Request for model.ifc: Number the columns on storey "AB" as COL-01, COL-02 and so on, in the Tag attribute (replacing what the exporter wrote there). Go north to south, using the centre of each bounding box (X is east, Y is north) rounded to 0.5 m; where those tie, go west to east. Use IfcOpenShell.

First a look at what the model holds.

```python
import ifcopenshell
import ifcopenshell.util.element
import ifcopenshell.util.placement

model = ifcopenshell.open("model.ifc")
print(model.schema)
storey = next(s for s in model.by_type("IfcBuildingStorey") if s.Name == "AB")
columns = [e for e in ifcopenshell.util.element.get_decomposition(storey) if e.is_a("IfcColumn")]
for e in sorted(columns, key=lambda e: e.id()):
    origin = ifcopenshell.util.placement.get_local_placement(e.ObjectPlacement)[:3, 3]
    print(e.id(), e.Tag, e.Name, origin.round(2) + 0.0, sep=" | ")
```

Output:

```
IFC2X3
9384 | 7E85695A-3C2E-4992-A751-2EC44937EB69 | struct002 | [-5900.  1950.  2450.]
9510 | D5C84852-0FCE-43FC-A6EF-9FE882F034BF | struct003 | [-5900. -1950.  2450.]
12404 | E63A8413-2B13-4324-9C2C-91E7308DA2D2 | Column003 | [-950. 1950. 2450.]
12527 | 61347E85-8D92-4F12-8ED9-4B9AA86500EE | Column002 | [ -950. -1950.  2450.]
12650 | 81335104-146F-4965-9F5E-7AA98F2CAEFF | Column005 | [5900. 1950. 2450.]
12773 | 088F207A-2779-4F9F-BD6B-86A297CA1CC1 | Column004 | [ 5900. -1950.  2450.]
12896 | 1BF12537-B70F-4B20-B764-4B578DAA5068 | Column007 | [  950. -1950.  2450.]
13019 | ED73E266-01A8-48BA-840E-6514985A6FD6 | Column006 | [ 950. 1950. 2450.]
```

```python
import ifcopenshell
import ifcopenshell.geom
import ifcopenshell.util.element
import ifcopenshell.util.shape

model = ifcopenshell.open("model.ifc")
settings = ifcopenshell.geom.settings()
settings.set("use-world-coords", True)


def centre(element):
    shape = ifcopenshell.geom.create_shape(settings, element)
    return ifcopenshell.util.shape.get_bbox_centroid(shape.geometry)


storey = next(s for s in model.by_type("IfcBuildingStorey") if s.Name == "AB")
columns = [e for e in ifcopenshell.util.element.get_decomposition(storey) if e.is_a("IfcColumn")]

# Insertion points can sit at a corner or the storey origin, so sort by the geometry (in metres).
centres = {e: centre(e) for e in columns}
columns.sort(key=lambda e: (-round(centres[e][1] / 0.5), centres[e][0]))

for i, e in enumerate(columns, start=1):
    number = f"COL-{i:02d}"
    e.Tag = number
    print(e.id(), number)

model.write("model_v2.ifc")
```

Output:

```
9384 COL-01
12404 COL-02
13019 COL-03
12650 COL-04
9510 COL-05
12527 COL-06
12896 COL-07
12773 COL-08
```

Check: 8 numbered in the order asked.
